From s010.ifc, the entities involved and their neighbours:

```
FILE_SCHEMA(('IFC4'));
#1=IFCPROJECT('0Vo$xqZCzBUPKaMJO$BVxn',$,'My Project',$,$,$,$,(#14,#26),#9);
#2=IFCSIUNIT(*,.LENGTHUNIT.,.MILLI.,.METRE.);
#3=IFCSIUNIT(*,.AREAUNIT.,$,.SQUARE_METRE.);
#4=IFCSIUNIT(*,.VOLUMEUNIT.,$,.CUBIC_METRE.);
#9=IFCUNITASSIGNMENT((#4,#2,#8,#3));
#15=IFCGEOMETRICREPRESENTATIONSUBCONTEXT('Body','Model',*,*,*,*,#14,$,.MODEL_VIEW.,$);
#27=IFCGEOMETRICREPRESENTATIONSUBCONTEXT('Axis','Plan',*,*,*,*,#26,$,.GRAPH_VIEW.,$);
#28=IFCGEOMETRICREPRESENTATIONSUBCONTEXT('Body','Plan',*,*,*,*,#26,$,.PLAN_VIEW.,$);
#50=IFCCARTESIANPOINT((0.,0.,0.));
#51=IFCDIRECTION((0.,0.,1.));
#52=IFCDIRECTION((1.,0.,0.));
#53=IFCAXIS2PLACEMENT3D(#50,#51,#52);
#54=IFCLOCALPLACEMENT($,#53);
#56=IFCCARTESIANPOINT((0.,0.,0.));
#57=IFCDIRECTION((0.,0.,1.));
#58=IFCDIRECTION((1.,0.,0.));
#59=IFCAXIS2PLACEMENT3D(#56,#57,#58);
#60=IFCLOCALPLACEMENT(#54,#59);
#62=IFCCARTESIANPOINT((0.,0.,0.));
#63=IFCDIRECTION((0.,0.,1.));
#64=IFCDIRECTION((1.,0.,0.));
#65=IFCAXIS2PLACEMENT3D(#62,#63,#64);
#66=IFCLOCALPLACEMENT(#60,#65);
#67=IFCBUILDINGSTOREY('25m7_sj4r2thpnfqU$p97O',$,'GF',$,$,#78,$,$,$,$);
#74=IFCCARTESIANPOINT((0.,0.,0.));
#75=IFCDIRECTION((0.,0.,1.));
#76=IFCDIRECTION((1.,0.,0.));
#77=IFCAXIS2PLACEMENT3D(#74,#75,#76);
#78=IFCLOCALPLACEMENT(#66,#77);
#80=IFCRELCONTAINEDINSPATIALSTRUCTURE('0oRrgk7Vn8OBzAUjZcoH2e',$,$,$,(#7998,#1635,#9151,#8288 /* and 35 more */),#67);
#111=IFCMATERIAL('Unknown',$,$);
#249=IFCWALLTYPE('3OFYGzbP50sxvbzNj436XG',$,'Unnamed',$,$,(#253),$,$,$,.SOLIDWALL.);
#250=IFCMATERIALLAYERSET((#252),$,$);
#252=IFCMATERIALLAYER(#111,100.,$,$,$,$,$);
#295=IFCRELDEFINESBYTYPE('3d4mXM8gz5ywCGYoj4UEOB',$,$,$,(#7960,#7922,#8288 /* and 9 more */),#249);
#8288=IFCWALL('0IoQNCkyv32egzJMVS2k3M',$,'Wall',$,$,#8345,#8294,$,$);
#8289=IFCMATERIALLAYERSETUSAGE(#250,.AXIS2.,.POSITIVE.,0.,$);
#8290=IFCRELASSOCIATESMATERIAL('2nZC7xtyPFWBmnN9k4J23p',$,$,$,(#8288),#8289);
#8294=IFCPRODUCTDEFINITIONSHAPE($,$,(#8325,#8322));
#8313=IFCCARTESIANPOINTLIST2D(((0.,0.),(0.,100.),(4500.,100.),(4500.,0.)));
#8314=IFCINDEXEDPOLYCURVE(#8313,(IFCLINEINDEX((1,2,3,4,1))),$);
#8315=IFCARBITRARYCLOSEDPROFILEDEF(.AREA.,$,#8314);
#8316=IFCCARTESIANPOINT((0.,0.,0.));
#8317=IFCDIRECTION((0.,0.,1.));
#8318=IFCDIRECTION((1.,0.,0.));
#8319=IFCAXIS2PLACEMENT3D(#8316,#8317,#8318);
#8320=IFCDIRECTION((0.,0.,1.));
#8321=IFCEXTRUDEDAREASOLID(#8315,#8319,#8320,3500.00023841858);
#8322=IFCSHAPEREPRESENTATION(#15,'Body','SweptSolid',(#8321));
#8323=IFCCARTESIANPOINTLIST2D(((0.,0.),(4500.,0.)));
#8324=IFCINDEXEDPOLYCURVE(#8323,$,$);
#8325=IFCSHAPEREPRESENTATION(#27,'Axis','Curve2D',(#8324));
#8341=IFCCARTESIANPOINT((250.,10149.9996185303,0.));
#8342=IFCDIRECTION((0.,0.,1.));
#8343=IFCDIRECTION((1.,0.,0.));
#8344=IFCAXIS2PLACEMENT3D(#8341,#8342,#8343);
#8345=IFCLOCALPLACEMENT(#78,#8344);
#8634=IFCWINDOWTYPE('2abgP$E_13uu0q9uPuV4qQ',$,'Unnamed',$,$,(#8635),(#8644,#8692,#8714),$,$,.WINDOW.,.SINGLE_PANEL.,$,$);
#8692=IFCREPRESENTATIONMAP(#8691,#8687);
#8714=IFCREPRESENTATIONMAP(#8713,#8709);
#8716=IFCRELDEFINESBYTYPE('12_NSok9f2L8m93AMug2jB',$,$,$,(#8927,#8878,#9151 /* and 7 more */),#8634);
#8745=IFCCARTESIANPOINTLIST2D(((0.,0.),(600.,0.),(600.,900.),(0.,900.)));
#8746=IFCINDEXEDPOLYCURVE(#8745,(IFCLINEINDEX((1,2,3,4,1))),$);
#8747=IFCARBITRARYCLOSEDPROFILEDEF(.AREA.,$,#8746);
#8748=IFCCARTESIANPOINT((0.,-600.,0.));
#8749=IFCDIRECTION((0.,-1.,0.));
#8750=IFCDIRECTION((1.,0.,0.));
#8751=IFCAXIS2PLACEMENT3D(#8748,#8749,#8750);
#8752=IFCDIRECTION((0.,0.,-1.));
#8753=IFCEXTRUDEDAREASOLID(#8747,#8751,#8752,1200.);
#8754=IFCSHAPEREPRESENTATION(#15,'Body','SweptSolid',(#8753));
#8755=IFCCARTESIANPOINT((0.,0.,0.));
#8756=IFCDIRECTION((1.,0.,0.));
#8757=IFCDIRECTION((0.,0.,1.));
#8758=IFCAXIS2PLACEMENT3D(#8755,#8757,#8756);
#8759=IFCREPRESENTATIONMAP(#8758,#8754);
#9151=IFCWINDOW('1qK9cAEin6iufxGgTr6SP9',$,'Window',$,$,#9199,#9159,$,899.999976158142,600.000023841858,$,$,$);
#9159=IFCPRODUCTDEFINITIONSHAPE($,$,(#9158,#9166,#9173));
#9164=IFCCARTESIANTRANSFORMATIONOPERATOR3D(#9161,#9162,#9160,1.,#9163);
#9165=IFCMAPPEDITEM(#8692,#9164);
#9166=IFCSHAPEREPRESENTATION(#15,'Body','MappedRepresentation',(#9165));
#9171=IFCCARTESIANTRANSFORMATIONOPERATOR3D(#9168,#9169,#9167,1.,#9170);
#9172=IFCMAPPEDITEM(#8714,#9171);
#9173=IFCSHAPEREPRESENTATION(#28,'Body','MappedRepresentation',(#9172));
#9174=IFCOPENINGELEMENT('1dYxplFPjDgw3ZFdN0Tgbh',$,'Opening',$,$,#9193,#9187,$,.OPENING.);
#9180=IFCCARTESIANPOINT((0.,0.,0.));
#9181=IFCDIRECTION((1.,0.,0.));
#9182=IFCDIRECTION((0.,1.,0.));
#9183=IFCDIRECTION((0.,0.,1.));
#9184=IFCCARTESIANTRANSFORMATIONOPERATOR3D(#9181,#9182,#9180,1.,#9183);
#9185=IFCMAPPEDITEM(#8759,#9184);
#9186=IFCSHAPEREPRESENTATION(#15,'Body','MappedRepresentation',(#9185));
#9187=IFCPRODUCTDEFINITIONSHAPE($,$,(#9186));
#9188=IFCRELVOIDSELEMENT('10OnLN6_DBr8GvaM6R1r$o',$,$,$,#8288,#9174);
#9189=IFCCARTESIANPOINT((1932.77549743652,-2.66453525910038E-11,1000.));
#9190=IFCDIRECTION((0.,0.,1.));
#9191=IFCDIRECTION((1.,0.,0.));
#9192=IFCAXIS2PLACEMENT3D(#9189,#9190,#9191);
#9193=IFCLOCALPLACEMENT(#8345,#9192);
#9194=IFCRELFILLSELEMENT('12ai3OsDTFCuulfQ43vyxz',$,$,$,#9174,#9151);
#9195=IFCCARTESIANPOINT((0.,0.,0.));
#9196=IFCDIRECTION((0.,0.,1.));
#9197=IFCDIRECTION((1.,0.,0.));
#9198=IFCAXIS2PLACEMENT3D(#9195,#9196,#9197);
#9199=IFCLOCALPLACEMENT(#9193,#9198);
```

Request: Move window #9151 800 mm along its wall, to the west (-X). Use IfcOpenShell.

```python
import ifcopenshell
import ifcopenshell.api.geometry
import ifcopenshell.util.placement
import ifcopenshell.util.unit

model = ifcopenshell.open("s010.ifc")
unit_scale = ifcopenshell.util.unit.calculate_unit_scale(model)

window = model.by_guid("1qK9cAEin6iufxGgTr6SP9")
opening = window.FillsVoids[0].RelatingOpeningElement
wall = opening.VoidsElements[0].RelatingBuildingElement

wall_matrix = ifcopenshell.util.placement.get_local_placement(wall.ObjectPlacement)
shift = wall_matrix[:3, 0] * -0.8 / unit_scale
before = ifcopenshell.util.placement.get_local_placement(window.ObjectPlacement)[:3, 3].copy()

# The window is placed relative to its opening, so it follows when the opening moves.
matrix = ifcopenshell.util.placement.get_local_placement(opening.ObjectPlacement)
matrix[:3, 3] += shift
ifcopenshell.api.geometry.edit_object_placement(
    model, product=opening, matrix=matrix, is_si=False, should_transform_children=True
)

after = ifcopenshell.util.placement.get_local_placement(window.ObjectPlacement)[:3, 3]
print("window moved by", (after - before).round(3) + 0.0)

model.write("s010-out.ifc")
```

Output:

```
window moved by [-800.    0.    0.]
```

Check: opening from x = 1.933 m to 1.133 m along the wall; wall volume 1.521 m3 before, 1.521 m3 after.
